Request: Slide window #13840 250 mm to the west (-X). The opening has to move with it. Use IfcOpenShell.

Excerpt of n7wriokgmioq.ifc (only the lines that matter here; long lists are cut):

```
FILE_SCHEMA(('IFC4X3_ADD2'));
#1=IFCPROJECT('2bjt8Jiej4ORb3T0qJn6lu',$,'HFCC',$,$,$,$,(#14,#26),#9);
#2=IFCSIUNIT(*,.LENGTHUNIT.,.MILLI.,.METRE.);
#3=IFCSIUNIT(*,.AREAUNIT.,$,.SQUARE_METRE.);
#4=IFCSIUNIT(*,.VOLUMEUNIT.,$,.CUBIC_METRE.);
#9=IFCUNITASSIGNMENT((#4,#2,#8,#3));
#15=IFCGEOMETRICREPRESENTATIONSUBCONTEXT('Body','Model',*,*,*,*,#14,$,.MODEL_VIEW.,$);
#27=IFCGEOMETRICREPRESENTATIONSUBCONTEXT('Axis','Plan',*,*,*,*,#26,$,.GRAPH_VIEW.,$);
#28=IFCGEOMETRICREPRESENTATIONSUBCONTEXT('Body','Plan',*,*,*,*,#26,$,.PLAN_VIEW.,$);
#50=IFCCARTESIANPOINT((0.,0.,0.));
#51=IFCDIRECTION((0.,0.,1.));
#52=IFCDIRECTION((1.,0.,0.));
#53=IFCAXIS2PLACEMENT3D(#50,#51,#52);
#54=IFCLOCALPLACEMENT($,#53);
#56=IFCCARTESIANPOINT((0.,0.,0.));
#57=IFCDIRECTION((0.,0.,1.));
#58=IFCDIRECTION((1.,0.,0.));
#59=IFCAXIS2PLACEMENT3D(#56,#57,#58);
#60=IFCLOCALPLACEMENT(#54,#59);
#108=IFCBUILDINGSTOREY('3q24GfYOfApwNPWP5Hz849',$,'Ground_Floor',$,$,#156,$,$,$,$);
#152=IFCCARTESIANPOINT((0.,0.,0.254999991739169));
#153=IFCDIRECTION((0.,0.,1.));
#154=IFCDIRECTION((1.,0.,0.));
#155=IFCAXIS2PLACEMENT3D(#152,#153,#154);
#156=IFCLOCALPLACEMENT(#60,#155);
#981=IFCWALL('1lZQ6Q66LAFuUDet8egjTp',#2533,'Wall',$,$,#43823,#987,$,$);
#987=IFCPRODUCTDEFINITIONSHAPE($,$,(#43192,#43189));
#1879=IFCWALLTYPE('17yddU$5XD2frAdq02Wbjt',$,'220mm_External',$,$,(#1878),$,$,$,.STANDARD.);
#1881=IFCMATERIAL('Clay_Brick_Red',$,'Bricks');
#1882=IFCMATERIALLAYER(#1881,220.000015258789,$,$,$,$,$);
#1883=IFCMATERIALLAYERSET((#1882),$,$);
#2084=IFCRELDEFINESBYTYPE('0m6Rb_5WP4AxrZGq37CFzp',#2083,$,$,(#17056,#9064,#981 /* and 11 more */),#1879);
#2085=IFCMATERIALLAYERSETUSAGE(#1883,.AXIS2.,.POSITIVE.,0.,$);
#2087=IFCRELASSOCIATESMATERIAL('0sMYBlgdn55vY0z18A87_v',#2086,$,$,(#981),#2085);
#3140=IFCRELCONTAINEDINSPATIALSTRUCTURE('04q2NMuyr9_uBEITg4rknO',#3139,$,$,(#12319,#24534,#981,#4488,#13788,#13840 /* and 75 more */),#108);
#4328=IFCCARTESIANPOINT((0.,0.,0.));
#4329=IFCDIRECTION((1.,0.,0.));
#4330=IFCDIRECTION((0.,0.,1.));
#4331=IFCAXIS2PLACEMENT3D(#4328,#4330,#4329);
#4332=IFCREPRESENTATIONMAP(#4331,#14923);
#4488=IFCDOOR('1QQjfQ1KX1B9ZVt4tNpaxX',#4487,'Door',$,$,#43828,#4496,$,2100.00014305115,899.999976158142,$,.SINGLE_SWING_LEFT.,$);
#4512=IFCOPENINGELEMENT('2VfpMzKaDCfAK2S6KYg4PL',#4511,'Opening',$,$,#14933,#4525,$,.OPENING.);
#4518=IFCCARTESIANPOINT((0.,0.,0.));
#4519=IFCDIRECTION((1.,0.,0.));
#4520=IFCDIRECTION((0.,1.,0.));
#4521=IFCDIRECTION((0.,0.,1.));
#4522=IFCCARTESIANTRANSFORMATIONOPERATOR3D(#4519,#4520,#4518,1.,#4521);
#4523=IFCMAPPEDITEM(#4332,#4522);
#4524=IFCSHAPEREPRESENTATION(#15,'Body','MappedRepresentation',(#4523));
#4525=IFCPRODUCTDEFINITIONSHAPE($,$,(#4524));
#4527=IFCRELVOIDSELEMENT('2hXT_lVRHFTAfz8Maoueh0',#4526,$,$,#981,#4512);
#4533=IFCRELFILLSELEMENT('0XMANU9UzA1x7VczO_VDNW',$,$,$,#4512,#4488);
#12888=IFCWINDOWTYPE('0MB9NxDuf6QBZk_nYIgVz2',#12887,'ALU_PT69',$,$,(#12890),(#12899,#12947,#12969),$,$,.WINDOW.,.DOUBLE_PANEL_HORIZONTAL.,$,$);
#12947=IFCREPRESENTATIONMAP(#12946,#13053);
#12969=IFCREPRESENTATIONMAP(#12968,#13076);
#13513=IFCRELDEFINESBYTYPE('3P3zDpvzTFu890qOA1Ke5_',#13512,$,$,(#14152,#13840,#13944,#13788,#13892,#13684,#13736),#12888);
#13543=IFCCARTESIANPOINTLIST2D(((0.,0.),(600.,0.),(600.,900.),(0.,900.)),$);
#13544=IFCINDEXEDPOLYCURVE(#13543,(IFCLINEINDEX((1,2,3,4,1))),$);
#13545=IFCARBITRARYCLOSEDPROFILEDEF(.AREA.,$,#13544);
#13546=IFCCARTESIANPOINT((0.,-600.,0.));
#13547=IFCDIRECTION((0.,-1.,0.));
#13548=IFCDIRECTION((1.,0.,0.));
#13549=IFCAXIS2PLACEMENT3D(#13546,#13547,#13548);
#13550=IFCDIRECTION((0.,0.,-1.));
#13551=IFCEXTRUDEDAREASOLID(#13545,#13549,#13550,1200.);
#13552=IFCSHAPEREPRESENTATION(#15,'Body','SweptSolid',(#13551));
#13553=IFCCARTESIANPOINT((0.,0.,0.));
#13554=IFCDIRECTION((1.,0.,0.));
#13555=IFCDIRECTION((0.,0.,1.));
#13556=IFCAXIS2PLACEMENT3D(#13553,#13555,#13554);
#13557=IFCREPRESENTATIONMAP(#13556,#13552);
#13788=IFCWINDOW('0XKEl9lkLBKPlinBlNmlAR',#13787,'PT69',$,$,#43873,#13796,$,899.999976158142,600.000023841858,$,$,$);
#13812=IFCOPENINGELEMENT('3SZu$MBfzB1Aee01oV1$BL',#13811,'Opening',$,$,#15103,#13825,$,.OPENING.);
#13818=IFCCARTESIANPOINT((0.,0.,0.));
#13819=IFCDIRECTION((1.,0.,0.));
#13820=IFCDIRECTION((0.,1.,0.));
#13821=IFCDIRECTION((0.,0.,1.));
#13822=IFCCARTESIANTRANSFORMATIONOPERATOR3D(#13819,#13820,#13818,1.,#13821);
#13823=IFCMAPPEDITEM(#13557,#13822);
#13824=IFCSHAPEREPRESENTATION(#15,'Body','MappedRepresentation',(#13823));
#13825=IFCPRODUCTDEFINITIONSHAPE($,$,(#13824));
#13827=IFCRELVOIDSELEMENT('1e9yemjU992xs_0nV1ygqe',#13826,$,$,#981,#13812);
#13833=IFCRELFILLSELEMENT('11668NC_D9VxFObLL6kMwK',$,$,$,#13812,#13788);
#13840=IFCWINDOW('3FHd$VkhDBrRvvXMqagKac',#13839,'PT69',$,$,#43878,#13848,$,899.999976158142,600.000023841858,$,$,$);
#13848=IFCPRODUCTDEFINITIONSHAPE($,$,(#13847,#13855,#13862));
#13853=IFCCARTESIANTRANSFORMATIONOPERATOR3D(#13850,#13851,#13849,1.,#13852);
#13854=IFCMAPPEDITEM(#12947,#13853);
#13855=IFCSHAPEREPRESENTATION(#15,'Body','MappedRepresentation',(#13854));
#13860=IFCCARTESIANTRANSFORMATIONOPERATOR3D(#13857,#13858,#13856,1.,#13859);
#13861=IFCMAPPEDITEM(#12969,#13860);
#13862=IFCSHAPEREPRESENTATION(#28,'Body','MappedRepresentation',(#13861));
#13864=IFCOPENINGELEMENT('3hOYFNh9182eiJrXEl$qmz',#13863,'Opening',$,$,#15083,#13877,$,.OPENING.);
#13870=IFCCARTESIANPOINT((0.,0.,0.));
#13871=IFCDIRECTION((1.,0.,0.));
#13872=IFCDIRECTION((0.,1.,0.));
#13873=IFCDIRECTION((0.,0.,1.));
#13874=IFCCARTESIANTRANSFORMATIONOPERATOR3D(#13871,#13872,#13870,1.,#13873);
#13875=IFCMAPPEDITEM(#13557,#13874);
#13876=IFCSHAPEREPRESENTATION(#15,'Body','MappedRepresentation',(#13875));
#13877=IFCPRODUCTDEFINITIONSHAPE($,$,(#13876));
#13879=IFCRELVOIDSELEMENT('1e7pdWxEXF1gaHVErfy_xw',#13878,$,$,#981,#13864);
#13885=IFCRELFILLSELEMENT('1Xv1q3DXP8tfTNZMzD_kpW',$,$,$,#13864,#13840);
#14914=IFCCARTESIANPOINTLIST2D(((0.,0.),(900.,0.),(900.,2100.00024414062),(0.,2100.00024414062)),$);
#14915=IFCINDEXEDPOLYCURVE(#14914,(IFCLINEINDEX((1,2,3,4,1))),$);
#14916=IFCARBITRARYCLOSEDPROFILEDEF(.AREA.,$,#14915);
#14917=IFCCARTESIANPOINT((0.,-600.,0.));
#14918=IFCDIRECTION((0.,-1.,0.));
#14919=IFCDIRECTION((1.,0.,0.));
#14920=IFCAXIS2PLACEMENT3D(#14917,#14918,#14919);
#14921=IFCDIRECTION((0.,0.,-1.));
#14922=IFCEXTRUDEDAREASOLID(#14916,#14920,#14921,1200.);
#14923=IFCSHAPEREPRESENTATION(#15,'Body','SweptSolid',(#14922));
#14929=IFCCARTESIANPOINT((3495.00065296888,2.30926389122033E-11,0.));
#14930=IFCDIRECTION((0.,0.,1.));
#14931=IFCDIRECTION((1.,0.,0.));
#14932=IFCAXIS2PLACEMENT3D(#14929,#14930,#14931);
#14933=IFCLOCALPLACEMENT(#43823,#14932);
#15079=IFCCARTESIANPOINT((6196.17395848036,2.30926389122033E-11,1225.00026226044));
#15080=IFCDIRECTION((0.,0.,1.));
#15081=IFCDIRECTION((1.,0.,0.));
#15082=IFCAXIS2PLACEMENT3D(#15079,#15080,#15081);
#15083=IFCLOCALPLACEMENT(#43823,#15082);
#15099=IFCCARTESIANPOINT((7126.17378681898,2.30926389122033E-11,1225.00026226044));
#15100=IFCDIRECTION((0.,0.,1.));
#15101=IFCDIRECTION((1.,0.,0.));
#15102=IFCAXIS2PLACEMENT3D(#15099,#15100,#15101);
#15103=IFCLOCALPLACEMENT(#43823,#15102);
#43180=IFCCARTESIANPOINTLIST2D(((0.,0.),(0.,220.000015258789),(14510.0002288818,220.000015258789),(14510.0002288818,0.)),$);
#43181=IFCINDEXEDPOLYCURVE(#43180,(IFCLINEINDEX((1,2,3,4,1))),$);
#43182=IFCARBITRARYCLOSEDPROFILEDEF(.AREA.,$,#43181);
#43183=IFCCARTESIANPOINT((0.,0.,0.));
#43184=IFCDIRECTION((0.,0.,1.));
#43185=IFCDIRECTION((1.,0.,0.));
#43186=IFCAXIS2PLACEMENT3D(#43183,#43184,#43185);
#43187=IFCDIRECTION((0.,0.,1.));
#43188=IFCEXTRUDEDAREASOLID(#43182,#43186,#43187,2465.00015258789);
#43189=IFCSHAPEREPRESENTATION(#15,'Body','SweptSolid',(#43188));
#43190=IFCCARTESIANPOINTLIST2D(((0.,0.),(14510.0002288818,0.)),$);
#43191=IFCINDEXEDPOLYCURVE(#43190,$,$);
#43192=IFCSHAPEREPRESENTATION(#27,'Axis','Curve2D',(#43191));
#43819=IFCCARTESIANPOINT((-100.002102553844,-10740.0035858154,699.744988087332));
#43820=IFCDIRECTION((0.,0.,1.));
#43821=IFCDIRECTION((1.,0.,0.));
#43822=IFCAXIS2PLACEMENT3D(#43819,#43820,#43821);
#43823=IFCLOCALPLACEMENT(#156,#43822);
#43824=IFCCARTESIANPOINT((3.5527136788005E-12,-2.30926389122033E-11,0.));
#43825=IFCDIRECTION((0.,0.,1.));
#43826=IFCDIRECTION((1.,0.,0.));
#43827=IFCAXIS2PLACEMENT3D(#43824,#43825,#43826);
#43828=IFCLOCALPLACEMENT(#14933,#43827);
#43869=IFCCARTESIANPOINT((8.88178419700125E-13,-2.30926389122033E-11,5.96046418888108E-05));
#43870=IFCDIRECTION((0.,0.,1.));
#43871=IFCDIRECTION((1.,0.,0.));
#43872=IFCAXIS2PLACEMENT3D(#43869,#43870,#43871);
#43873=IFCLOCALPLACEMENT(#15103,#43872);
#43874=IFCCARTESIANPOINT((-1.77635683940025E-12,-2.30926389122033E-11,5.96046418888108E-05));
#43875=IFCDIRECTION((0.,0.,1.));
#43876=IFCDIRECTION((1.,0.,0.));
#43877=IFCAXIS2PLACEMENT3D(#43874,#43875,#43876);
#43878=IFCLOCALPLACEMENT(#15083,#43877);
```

```python
import ifcopenshell
import ifcopenshell.api.geometry
import ifcopenshell.util.placement
import ifcopenshell.util.unit

model = ifcopenshell.open("n7wriokgmioq.ifc")
unit_scale = ifcopenshell.util.unit.calculate_unit_scale(model)

window = model.by_guid("3FHd$VkhDBrRvvXMqagKac")
opening = window.FillsVoids[0].RelatingOpeningElement
wall = opening.VoidsElements[0].RelatingBuildingElement

wall_matrix = ifcopenshell.util.placement.get_local_placement(wall.ObjectPlacement)
shift = wall_matrix[:3, 0] * -0.25 / unit_scale
before = ifcopenshell.util.placement.get_local_placement(window.ObjectPlacement)[:3, 3].copy()

# The window is placed relative to its opening, so it follows when the opening moves.
matrix = ifcopenshell.util.placement.get_local_placement(opening.ObjectPlacement)
matrix[:3, 3] += shift
ifcopenshell.api.geometry.edit_object_placement(
    model, product=opening, matrix=matrix, is_si=False, should_transform_children=True
)

after = ifcopenshell.util.placement.get_local_placement(window.ObjectPlacement)[:3, 3]
print("window moved by", (after - before).round(3) + 0.0)

model.write("n7wriokgmioq_edited.ifc")
```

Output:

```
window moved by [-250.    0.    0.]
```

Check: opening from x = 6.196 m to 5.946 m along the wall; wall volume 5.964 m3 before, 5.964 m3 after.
